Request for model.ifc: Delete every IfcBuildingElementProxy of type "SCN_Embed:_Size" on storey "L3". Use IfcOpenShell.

First a look at what the model holds.

```python
import ifcopenshell
import ifcopenshell.util.element

model = ifcopenshell.open("model.ifc")
print(model.schema)
storey = next(s for s in model.by_type("IfcBuildingStorey") if s.Name == "L3")
proxies = [e for e in ifcopenshell.util.element.get_decomposition(storey) if e.is_a("IfcBuildingElementProxy")]
seen = {}
for e in proxies:
    element_type = ifcopenshell.util.element.get_type(e)
    name = element_type.Name if element_type not in (None, e) else None
    seen[name] = seen.get(name, 0) + 1
for name, count in sorted(seen.items(), key=str):
    print(count, "x", name)
```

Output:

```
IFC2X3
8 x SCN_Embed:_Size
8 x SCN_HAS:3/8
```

```python
import ifcopenshell
import ifcopenshell.api.root
import ifcopenshell.util.element

model = ifcopenshell.open("model.ifc")

storey = next(s for s in model.by_type("IfcBuildingStorey") if s.Name == "L3")
proxies = [e for e in ifcopenshell.util.element.get_decomposition(storey) if e.is_a("IfcBuildingElementProxy")]
targets = [e for e in proxies if (t := ifcopenshell.util.element.get_type(e)) not in (None, e) and t.Name == "SCN_Embed:_Size"]

for e in targets:
    ifcopenshell.api.root.remove_product(model, product=e)
print(len(targets), "removed")

model.write("model_updated.ifc")
```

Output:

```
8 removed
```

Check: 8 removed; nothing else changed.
